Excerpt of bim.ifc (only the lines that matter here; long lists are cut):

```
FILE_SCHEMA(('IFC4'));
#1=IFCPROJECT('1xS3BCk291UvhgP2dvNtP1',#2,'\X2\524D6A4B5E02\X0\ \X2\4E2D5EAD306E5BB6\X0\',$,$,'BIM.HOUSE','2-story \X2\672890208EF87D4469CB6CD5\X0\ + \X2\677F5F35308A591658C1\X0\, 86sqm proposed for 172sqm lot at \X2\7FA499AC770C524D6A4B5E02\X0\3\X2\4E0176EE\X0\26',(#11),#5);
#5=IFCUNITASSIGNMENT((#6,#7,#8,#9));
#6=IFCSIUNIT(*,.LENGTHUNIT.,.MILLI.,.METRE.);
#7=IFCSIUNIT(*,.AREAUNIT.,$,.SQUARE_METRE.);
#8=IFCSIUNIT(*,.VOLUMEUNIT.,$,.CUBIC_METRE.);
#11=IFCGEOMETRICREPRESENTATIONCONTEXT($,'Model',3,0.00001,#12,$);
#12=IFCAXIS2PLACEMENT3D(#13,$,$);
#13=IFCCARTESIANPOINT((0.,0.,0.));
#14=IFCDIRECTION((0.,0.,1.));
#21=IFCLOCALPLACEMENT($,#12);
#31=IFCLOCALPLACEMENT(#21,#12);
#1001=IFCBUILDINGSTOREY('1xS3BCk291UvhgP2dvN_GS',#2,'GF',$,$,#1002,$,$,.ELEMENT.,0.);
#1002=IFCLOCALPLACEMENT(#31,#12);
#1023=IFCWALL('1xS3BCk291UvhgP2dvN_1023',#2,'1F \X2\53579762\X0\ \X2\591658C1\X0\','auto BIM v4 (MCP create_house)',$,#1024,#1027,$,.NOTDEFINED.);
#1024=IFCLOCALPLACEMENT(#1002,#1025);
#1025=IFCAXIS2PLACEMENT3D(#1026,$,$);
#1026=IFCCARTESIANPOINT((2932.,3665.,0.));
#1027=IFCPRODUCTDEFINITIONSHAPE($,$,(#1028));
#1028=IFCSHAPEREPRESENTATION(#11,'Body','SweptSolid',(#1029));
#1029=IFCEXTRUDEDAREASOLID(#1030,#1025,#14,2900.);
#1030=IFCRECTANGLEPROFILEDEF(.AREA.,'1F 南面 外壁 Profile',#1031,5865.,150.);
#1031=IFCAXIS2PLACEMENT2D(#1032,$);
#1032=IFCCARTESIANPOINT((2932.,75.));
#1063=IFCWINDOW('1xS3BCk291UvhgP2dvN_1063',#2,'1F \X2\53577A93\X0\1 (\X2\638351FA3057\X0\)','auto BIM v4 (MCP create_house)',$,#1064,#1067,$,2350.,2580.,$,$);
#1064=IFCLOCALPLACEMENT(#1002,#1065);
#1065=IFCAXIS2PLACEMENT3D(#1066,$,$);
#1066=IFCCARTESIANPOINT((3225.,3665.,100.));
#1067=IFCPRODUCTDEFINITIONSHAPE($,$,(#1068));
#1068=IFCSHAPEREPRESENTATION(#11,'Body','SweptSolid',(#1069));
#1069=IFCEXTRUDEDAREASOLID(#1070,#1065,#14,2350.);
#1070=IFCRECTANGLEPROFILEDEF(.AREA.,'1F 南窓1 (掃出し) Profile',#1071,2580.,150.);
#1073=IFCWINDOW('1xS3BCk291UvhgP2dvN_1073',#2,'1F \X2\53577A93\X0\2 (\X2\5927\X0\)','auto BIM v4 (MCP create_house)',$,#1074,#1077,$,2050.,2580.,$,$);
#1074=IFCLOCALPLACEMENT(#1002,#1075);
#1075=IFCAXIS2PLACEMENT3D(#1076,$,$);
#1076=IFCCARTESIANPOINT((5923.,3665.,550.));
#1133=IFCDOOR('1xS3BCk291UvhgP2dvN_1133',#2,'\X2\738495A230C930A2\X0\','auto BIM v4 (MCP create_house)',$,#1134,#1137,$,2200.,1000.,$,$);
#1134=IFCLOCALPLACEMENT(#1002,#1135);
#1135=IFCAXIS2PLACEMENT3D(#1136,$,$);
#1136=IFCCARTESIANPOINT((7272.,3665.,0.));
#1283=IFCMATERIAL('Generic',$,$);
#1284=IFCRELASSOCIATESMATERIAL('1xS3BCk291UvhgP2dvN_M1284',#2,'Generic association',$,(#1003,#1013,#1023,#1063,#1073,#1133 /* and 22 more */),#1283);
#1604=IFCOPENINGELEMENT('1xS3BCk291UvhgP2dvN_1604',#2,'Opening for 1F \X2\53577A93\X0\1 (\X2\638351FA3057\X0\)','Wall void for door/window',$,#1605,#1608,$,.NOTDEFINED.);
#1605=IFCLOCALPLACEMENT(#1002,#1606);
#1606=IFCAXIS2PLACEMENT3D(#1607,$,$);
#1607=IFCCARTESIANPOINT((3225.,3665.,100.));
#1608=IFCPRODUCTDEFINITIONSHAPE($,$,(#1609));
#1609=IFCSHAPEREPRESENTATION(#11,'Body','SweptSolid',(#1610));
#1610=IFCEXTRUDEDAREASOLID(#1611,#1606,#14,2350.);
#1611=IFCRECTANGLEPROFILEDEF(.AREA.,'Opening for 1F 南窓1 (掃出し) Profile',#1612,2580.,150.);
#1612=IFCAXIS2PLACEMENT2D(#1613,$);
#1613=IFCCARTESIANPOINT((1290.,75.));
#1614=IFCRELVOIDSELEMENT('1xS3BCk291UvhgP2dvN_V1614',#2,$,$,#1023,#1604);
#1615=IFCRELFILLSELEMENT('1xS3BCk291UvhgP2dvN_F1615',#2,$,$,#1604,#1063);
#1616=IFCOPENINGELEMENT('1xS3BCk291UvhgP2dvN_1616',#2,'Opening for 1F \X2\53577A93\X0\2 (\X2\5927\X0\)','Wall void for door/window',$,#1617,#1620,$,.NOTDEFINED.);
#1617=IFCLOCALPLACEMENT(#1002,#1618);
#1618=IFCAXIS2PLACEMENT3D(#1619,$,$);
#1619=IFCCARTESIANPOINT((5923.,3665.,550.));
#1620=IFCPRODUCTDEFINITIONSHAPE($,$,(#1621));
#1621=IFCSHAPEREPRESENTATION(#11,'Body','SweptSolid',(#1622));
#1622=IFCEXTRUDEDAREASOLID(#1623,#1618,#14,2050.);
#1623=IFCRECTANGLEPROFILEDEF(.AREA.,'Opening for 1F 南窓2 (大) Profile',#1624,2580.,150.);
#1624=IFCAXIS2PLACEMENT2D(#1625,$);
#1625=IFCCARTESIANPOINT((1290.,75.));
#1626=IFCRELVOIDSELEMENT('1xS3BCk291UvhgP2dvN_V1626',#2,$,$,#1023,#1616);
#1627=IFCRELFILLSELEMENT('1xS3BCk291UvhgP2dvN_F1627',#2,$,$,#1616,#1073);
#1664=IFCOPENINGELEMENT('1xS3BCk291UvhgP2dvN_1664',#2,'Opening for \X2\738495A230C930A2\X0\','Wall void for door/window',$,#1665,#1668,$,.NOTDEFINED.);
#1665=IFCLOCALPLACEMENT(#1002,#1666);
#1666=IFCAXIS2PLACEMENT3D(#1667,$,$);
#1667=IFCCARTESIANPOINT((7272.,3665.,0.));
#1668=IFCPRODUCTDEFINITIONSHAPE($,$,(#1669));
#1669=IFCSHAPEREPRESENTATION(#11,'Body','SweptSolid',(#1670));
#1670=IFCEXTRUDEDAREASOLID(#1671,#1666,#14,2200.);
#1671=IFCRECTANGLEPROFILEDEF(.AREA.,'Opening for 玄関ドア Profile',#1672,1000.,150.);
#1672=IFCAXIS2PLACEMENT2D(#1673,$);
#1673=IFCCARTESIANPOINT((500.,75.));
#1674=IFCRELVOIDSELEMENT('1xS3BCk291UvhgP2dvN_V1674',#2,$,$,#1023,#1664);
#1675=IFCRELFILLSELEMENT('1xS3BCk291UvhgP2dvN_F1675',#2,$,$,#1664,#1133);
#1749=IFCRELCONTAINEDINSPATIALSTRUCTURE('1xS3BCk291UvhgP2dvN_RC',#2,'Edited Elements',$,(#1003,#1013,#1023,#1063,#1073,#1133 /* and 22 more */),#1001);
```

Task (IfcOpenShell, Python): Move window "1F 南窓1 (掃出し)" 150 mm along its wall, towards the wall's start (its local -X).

```python
import ifcopenshell
import ifcopenshell.api.geometry
import ifcopenshell.util.placement
import ifcopenshell.util.unit

model = ifcopenshell.open("bim.ifc")
unit_scale = ifcopenshell.util.unit.calculate_unit_scale(model)

window = model.by_guid("1xS3BCk291UvhgP2dvN_1063")
opening = window.FillsVoids[0].RelatingOpeningElement
wall = opening.VoidsElements[0].RelatingBuildingElement

wall_matrix = ifcopenshell.util.placement.get_local_placement(wall.ObjectPlacement)
shift = wall_matrix[:3, 0] * -0.15 / unit_scale
before = ifcopenshell.util.placement.get_local_placement(window.ObjectPlacement)[:3, 3].copy()

# The window is not placed relative to its opening, so move both.
for product in (opening, window):
    matrix = ifcopenshell.util.placement.get_local_placement(product.ObjectPlacement)
    matrix[:3, 3] += shift
    ifcopenshell.api.geometry.edit_object_placement(model, product=product, matrix=matrix, is_si=False)

after = ifcopenshell.util.placement.get_local_placement(window.ObjectPlacement)[:3, 3]
print("window moved by", (after - before).round(3) + 0.0)

model.write("bim-out.ifc")
```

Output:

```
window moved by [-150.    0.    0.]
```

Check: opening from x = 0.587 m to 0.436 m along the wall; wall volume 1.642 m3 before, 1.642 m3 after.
